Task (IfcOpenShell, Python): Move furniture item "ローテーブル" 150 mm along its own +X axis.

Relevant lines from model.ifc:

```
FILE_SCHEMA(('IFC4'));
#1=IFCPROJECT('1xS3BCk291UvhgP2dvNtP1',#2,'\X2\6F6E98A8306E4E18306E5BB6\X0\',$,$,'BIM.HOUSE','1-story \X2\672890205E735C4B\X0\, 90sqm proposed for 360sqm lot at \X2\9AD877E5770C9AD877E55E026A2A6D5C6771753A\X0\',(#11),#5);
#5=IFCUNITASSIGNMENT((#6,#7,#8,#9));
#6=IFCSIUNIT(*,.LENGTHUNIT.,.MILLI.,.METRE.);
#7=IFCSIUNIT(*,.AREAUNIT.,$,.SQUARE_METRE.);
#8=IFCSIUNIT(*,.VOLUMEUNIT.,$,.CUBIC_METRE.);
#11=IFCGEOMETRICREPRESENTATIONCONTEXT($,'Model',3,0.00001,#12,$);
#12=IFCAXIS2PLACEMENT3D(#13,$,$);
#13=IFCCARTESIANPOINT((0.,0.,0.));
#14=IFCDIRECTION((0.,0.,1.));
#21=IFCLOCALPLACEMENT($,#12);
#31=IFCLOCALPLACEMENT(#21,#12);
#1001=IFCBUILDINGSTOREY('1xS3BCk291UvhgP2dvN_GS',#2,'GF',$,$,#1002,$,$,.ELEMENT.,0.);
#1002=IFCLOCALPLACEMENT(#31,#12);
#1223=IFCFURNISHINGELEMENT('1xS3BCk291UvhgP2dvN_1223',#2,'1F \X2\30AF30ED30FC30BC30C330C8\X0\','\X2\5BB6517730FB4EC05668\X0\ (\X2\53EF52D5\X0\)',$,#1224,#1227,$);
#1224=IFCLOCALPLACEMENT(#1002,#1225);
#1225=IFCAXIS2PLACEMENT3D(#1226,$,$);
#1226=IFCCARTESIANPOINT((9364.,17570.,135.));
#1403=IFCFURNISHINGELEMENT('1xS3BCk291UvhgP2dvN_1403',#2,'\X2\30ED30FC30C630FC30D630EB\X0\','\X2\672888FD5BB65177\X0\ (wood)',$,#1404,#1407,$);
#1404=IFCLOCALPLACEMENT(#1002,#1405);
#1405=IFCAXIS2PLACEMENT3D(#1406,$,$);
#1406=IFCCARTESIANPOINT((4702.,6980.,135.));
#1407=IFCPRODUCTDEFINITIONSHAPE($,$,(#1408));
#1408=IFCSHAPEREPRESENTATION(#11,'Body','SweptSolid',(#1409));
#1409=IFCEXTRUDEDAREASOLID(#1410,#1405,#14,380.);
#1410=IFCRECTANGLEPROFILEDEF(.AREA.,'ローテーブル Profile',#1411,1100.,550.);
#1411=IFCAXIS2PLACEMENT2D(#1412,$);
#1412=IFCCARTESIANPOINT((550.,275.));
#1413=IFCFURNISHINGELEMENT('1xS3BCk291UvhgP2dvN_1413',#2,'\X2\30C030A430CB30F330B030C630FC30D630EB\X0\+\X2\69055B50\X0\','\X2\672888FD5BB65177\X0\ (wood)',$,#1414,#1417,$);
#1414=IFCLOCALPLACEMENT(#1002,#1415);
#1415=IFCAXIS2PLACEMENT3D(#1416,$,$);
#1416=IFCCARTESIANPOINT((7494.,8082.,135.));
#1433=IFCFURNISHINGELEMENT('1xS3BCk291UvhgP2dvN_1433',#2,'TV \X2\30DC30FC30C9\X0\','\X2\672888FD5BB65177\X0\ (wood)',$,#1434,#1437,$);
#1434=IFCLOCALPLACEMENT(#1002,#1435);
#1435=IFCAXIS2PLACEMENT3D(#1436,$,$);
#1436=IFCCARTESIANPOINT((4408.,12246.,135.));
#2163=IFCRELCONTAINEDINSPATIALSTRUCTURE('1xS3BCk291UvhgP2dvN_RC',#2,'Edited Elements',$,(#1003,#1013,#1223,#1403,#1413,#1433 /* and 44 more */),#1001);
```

```python
import ifcopenshell
import ifcopenshell.api.geometry
import ifcopenshell.util.placement
import ifcopenshell.util.unit

model = ifcopenshell.open("model.ifc")
unit_scale = ifcopenshell.util.unit.calculate_unit_scale(model)

item = model.by_guid("1xS3BCk291UvhgP2dvN_1403")
matrix = ifcopenshell.util.placement.get_local_placement(item.ObjectPlacement)
matrix[:3, 3] += matrix[:3, 0] * 0.15 / unit_scale
ifcopenshell.api.geometry.edit_object_placement(model, product=item, matrix=matrix, is_si=False)

print(ifcopenshell.util.placement.get_local_placement(item.ObjectPlacement).round(3) + 0.0)

model.write("model-out.ifc")
```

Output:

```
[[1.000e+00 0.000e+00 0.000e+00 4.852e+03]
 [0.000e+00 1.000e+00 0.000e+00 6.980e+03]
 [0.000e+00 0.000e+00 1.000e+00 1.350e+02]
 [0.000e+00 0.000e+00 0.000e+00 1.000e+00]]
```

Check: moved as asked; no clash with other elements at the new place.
